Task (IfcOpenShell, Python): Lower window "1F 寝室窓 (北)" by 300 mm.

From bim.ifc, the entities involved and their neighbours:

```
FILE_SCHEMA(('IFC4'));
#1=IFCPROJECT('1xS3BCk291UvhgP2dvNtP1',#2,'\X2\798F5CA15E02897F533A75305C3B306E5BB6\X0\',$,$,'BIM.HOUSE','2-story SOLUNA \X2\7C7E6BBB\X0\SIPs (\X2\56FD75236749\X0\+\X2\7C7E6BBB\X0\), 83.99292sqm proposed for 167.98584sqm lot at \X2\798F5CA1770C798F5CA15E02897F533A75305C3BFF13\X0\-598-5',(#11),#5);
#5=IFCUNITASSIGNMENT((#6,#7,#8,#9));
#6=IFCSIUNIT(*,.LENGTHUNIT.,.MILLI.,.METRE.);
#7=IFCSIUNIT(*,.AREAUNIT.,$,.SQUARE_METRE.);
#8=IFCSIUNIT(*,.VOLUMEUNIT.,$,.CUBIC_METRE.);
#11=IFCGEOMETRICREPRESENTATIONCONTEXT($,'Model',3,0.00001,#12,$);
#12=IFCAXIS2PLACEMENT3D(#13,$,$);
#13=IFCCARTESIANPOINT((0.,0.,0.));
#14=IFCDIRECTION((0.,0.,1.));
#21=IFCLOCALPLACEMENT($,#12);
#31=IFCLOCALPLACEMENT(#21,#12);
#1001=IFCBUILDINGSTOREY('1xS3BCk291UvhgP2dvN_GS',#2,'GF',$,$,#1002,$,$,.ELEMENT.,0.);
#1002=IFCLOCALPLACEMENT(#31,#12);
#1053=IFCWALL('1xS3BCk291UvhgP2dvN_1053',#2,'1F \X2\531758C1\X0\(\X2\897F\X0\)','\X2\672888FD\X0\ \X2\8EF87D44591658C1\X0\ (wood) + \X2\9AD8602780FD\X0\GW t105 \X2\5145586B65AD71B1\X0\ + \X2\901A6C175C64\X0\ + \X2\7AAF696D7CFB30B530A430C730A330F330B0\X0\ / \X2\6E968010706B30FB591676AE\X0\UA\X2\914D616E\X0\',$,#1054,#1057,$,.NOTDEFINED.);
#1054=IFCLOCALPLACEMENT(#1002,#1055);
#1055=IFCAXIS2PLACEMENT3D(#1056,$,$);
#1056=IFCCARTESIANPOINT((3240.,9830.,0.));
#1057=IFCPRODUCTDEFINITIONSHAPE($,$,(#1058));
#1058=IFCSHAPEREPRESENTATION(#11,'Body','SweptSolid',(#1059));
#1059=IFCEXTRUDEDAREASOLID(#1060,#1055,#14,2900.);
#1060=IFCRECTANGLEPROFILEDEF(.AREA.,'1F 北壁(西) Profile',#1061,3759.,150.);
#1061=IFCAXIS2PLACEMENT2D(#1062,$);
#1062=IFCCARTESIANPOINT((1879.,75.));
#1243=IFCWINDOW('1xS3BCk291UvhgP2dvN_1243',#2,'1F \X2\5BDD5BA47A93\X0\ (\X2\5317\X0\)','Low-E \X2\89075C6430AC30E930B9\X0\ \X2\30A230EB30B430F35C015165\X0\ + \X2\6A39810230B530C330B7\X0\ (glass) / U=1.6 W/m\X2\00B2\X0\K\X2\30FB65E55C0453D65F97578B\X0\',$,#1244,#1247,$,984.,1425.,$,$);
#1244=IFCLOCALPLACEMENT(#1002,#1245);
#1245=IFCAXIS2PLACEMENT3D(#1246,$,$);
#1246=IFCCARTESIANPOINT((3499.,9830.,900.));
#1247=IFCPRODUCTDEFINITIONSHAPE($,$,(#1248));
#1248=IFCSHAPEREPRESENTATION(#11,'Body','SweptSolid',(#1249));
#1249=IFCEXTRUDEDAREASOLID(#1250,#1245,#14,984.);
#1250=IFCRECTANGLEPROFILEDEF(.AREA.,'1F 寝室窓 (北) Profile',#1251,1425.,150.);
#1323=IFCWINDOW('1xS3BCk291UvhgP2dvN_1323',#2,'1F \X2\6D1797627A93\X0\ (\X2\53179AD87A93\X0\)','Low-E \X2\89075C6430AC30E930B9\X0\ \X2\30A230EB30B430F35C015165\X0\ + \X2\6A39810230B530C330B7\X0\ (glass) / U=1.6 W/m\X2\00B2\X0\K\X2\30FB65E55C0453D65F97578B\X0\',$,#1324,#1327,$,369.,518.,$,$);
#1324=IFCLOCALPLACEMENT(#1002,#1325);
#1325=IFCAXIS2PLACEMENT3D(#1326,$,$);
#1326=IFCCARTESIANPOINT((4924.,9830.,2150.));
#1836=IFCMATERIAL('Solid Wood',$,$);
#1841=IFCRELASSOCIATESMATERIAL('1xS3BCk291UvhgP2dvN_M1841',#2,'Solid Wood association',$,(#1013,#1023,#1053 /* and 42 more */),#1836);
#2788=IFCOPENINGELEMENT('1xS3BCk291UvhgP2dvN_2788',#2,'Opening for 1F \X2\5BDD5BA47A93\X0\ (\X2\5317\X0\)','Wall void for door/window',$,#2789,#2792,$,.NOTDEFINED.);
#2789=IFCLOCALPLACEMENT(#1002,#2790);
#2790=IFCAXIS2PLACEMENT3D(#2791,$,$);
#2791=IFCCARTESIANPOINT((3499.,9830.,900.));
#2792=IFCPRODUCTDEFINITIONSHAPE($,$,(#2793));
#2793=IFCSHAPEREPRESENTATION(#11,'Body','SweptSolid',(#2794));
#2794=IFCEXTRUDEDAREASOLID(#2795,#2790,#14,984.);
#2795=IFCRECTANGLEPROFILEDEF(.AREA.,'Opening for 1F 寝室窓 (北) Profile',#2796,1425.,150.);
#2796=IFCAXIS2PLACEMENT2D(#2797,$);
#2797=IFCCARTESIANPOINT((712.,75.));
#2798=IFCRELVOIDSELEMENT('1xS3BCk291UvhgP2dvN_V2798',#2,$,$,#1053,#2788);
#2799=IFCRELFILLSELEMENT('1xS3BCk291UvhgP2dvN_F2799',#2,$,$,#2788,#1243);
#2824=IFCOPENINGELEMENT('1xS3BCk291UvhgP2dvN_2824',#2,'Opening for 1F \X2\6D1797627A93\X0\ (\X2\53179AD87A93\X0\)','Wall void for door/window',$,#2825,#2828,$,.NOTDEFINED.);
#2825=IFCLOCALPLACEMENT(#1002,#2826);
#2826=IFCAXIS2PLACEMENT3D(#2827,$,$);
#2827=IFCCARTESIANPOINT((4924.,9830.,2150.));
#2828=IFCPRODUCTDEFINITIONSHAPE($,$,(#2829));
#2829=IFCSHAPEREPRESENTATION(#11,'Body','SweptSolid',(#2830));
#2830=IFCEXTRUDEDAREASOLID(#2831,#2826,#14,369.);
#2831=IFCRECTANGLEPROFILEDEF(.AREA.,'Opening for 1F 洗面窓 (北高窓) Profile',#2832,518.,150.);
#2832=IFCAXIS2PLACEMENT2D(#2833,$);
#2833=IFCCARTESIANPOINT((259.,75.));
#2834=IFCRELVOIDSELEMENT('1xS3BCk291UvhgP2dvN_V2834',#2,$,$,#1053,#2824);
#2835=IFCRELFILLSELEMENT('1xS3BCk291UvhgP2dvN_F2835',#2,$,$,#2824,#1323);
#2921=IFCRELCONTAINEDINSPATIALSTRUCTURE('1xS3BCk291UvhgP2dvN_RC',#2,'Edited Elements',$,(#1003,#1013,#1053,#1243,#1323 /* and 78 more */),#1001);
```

```python
import numpy as np
import ifcopenshell
import ifcopenshell.api.geometry
import ifcopenshell.util.placement
import ifcopenshell.util.unit

model = ifcopenshell.open("bim.ifc")
unit_scale = ifcopenshell.util.unit.calculate_unit_scale(model)

window = model.by_id(1243)
opening = window.FillsVoids[0].RelatingOpeningElement
dz = -0.3 / unit_scale

shift = np.array([0.0, 0.0, dz])
# The window is not placed relative to its opening, so move both.
for product in (opening, window):
    matrix = ifcopenshell.util.placement.get_local_placement(product.ObjectPlacement)
    matrix[:3, 3] += shift
    ifcopenshell.api.geometry.edit_object_placement(model, product=product, matrix=matrix, is_si=False)

print(f"moved by {dz * unit_scale:+.3f} m")

model.write("bim_v2.ifc")
```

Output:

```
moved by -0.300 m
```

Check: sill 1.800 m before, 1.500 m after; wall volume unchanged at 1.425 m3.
